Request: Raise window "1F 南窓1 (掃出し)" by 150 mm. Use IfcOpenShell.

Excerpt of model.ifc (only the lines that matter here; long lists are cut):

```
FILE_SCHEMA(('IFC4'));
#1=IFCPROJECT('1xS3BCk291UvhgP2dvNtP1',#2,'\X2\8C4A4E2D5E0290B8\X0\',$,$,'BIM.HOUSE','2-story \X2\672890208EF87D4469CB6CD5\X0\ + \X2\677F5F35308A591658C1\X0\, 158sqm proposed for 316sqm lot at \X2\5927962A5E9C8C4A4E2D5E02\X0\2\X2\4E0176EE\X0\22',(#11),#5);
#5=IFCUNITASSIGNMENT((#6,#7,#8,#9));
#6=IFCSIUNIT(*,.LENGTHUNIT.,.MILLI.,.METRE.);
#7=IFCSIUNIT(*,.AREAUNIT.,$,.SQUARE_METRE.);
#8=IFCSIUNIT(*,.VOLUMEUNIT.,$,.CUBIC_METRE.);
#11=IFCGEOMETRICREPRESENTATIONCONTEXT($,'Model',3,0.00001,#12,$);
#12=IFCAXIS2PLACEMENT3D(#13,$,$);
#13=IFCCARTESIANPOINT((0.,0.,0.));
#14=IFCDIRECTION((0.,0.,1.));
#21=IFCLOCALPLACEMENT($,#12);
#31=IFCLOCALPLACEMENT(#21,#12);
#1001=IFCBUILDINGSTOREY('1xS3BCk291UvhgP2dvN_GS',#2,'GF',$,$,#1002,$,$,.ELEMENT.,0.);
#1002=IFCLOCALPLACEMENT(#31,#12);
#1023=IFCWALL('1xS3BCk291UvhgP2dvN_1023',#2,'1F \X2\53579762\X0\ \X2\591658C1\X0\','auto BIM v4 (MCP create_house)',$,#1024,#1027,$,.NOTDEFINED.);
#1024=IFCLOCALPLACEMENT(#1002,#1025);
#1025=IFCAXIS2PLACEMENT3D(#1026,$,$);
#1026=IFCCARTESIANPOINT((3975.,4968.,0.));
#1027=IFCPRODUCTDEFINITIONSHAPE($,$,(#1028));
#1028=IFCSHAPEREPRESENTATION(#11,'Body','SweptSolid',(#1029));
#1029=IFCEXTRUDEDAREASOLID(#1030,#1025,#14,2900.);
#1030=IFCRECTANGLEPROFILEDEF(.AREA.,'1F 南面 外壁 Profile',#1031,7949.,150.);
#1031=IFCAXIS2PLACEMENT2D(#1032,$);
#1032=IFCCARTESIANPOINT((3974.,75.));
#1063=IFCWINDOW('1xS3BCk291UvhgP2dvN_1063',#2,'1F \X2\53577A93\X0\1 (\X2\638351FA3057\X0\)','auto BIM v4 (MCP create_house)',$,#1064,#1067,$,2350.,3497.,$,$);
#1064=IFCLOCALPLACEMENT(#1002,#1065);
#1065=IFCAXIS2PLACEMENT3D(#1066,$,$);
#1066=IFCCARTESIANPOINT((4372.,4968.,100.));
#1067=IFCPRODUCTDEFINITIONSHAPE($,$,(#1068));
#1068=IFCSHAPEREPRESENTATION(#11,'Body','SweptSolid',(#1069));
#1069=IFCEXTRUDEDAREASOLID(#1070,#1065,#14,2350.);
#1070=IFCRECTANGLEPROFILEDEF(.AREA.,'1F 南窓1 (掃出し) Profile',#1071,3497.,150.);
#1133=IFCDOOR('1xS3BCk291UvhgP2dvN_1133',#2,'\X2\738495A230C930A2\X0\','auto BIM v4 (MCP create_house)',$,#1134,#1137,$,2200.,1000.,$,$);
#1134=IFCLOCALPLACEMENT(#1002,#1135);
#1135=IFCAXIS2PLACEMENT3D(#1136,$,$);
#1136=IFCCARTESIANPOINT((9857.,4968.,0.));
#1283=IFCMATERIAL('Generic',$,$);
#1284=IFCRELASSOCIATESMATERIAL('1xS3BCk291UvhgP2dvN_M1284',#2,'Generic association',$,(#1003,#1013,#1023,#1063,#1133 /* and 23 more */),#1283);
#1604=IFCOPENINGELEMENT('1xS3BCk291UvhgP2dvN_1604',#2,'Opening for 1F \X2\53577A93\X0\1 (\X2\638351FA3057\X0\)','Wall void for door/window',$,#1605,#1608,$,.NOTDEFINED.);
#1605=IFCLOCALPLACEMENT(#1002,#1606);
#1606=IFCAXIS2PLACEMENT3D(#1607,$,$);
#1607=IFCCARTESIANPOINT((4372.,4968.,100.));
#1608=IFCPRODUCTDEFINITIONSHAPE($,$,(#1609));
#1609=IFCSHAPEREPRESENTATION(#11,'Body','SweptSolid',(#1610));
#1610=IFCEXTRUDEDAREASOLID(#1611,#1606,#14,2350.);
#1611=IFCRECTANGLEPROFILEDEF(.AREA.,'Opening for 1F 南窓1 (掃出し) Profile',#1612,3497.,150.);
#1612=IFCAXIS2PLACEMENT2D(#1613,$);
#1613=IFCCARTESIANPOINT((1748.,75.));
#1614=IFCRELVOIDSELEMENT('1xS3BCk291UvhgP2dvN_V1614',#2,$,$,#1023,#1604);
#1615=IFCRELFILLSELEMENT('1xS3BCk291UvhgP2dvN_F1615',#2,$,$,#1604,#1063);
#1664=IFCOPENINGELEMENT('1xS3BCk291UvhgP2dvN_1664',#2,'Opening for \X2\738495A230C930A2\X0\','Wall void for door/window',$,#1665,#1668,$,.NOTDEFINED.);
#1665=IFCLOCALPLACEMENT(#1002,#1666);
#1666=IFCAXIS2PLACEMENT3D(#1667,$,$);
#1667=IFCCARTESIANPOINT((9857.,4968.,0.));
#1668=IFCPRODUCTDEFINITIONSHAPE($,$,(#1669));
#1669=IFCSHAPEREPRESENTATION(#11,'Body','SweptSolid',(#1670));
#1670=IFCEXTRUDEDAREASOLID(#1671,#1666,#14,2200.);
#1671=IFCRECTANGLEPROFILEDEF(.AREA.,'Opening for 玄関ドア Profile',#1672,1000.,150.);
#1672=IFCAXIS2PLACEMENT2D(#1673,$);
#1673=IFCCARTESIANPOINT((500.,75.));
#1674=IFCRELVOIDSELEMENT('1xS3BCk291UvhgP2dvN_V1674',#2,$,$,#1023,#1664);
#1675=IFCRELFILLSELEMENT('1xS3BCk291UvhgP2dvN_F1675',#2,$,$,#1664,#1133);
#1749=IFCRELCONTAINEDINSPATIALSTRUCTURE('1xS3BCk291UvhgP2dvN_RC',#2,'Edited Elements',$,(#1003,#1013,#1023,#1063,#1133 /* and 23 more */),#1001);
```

```python
import numpy as np
import ifcopenshell
import ifcopenshell.api.geometry
import ifcopenshell.util.placement
import ifcopenshell.util.unit

model = ifcopenshell.open("model.ifc")
unit_scale = ifcopenshell.util.unit.calculate_unit_scale(model)

window = model.by_guid("1xS3BCk291UvhgP2dvN_1063")
opening = window.FillsVoids[0].RelatingOpeningElement
dz = 150.0

shift = np.array([0.0, 0.0, dz])
# The window is not placed relative to its opening, so move both.
for product in (opening, window):
    matrix = ifcopenshell.util.placement.get_local_placement(product.ObjectPlacement)
    matrix[:3, 3] += shift
    ifcopenshell.api.geometry.edit_object_placement(model, product=product, matrix=matrix, is_si=False)

print(f"moved by {dz * unit_scale:+.3f} m")

model.write("model_v2.ifc")
```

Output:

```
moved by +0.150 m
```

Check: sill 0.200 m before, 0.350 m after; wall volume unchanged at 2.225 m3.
